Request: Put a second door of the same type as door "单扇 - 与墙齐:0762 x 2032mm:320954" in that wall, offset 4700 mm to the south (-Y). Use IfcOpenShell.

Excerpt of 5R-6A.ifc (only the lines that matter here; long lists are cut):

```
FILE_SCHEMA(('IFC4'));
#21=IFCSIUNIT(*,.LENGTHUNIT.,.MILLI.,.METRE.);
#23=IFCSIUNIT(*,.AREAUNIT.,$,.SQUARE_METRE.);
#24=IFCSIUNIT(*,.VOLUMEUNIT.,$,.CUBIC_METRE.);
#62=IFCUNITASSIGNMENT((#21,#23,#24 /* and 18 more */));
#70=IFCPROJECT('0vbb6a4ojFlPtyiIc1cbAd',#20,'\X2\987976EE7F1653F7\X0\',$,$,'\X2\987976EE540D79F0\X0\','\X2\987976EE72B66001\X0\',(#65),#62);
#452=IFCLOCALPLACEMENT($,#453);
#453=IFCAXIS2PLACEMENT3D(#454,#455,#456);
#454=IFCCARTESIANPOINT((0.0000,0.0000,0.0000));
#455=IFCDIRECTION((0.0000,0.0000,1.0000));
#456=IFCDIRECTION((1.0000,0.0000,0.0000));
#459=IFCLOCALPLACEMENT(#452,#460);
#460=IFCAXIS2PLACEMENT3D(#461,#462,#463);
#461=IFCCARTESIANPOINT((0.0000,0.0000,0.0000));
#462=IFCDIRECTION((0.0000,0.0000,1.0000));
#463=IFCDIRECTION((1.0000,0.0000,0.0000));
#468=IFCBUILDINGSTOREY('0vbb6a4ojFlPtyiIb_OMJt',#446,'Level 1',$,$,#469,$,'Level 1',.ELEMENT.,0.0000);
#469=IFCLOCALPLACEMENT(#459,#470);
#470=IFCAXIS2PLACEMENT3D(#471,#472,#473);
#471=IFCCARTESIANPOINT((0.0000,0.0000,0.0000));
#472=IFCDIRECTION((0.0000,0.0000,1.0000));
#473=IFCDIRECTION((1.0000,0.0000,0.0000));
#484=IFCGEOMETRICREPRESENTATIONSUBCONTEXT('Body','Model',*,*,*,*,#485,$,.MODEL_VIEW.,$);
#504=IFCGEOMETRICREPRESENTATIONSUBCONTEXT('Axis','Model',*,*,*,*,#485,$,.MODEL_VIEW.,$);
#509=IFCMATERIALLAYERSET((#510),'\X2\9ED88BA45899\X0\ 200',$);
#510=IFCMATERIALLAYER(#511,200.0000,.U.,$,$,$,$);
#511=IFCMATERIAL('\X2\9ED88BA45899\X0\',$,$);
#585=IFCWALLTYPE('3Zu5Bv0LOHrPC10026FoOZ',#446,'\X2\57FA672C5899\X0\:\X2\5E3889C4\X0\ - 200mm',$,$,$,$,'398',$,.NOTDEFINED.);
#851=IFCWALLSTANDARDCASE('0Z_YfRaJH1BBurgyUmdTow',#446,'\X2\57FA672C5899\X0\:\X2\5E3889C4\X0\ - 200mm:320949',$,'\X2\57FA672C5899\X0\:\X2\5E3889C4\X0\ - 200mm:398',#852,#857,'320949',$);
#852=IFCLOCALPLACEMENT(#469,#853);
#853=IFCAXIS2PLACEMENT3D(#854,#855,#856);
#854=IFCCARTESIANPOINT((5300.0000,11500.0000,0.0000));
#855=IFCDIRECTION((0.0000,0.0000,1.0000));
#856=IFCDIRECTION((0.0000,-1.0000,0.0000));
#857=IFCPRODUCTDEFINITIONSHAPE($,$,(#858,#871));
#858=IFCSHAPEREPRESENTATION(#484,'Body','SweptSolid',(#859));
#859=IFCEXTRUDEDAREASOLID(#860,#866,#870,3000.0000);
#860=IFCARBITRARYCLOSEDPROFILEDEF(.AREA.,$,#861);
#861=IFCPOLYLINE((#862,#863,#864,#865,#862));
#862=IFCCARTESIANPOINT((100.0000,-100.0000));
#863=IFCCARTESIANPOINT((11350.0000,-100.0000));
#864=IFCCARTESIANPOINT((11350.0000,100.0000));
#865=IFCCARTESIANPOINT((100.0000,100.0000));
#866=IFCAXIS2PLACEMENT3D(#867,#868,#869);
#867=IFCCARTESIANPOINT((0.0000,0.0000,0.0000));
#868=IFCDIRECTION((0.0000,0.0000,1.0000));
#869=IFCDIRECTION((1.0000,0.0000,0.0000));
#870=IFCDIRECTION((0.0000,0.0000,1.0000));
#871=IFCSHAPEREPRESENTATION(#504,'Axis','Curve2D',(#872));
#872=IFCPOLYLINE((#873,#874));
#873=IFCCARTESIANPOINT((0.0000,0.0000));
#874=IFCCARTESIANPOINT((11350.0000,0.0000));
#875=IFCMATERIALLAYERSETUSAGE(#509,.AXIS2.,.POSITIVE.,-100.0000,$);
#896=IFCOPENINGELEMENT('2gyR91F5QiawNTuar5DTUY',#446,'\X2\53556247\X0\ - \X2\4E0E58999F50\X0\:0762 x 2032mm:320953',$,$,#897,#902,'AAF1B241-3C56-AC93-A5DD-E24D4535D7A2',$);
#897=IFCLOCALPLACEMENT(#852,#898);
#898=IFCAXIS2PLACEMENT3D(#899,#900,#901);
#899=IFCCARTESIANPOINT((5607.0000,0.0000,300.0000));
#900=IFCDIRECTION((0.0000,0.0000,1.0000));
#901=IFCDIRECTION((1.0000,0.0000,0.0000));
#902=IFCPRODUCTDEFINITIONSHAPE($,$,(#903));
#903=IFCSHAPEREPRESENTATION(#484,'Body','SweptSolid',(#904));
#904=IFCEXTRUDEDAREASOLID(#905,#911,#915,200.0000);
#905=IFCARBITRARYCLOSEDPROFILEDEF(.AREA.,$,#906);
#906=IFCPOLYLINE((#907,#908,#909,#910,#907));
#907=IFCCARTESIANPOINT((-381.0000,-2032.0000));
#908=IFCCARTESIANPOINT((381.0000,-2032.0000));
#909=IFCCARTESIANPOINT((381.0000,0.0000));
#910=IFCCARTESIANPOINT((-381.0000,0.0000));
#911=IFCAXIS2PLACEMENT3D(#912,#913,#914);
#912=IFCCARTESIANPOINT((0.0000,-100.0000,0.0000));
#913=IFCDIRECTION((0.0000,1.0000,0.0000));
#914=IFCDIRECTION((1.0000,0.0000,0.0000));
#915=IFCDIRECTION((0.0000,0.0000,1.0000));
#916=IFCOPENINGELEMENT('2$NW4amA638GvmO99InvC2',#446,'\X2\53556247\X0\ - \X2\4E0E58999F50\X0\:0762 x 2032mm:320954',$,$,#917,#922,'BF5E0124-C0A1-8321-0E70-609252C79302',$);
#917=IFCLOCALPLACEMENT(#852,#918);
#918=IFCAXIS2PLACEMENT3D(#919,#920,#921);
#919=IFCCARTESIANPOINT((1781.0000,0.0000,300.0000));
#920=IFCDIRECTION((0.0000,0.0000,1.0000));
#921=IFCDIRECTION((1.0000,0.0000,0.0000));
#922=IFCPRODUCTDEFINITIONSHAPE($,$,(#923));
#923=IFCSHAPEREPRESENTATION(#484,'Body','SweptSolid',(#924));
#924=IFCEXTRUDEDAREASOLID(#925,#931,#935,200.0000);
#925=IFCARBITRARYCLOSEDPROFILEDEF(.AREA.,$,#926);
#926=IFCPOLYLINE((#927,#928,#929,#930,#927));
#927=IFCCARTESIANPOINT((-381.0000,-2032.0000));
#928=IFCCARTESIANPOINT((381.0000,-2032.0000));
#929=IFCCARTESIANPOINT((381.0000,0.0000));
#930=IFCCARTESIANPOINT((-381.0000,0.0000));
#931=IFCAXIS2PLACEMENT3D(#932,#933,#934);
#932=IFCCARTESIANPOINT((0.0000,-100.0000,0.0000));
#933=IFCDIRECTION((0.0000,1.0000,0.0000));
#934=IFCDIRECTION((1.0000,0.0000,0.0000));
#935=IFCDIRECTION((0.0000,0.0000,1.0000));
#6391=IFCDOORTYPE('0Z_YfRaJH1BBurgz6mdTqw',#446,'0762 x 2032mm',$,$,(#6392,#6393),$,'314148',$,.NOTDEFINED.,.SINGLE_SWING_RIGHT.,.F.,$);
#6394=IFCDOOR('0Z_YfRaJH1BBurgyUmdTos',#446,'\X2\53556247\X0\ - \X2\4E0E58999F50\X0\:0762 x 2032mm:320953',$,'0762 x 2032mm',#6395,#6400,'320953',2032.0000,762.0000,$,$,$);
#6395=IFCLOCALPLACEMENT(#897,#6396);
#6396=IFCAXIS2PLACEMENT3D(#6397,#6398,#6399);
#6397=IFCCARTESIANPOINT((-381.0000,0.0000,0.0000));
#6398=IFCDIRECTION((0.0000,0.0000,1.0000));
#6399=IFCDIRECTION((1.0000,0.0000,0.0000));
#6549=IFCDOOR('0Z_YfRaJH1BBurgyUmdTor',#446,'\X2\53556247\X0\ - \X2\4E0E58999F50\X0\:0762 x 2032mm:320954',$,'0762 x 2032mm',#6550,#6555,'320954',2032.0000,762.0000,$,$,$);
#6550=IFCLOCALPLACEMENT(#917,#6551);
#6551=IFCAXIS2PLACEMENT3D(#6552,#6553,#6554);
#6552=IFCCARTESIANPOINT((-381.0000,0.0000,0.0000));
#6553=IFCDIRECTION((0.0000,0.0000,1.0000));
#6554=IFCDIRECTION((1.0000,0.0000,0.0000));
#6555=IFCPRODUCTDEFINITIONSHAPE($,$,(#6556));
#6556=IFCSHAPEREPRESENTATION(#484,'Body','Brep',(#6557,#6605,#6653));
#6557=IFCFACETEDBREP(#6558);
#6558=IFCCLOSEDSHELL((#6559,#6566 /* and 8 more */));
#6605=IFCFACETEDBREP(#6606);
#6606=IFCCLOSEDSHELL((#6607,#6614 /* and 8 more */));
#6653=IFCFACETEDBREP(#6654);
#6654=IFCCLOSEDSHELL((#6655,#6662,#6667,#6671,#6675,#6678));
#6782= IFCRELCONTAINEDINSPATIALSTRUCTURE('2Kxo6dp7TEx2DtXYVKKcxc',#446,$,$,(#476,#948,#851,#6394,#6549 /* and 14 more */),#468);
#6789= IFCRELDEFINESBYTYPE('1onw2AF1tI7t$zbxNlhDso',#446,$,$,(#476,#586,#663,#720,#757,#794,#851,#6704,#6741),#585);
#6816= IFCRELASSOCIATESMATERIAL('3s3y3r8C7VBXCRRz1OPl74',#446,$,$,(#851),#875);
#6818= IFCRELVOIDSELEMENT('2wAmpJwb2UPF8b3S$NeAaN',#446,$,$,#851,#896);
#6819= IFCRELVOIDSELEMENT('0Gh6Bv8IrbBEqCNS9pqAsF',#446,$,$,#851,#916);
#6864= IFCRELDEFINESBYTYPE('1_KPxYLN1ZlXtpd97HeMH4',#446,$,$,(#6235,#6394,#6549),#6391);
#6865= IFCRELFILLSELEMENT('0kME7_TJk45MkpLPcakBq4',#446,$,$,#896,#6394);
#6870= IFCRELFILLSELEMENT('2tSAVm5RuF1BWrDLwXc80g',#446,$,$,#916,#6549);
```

```python
import ifcopenshell
import ifcopenshell.api.feature
import ifcopenshell.api.geometry
import ifcopenshell.api.root
import ifcopenshell.geom
import ifcopenshell.util.element
import ifcopenshell.util.placement
import ifcopenshell.util.shape
import ifcopenshell.util.unit

model = ifcopenshell.open("5R-6A.ifc")
unit_scale = ifcopenshell.util.unit.calculate_unit_scale(model)
settings = ifcopenshell.geom.settings()


def volume(element):
    """Net volume in cubic metres, openings subtracted."""
    shape = ifcopenshell.geom.create_shape(settings, element)
    return ifcopenshell.util.shape.get_volume(shape.geometry)


def reuse_history(source, copy):
    """copy_class also copies each property set's owner history, people and application; keep the originals."""
    for rel in copy.IsDefinedBy:
        if rel.is_a("IfcRelDefinesByProperties") and (history := rel.RelatingPropertyDefinition.OwnerHistory):
            rel.RelatingPropertyDefinition.OwnerHistory = source.OwnerHistory
            ifcopenshell.util.element.remove_deep2(model, history)


door = model.by_id(6549)
opening = door.FillsVoids[0].RelatingOpeningElement
wall = opening.VoidsElements[0].RelatingBuildingElement
before = volume(wall)
shift = ifcopenshell.util.placement.get_local_placement(wall.ObjectPlacement)[:3, 0] * 4.7 / unit_scale

# copy_class copies the void relationship, type, container and properties, but no geometry.
new_opening = ifcopenshell.api.root.copy_class(model, product=opening)
new_opening.Representation = ifcopenshell.util.element.copy_deep(
    model, opening.Representation, exclude=["IfcGeometricRepresentationContext", "IfcRepresentationMap"]
)
new_opening.Name = "单扇 - 与墙齐:0762 x 2032mm"
new_opening.Tag = None
new_door = ifcopenshell.api.root.copy_class(model, product=door)
new_door.Representation = ifcopenshell.util.element.copy_deep(
    model, door.Representation, exclude=["IfcGeometricRepresentationContext", "IfcRepresentationMap"]
)
new_door.Name = "单扇 - 与墙齐:0762 x 2032mm"
new_door.Tag = None
reuse_history(door, new_door)
ifcopenshell.api.feature.add_filling(model, opening=new_opening, element=new_door)

for old, new in ((opening, new_opening), (door, new_door)):
    matrix = ifcopenshell.util.placement.get_local_placement(old.ObjectPlacement)
    matrix[:3, 3] += shift
    ifcopenshell.api.geometry.edit_object_placement(model, product=new, matrix=matrix, is_si=False)

after = volume(wall)

print(f"wall volume {before:.3f} -> {after:.3f} m3")

model.write("5R-6A_edited.ifc")
```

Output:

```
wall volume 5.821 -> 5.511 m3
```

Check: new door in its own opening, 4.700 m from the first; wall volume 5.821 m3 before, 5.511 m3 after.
